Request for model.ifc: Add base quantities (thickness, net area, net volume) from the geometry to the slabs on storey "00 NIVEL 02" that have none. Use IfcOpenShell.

First a look at what the model holds.

```python
import ifcopenshell
import ifcopenshell.util.element
import ifcopenshell.util.unit

model = ifcopenshell.open("model.ifc")
print(model.schema)
for unit_type in ("LENGTHUNIT", "AREAUNIT", "VOLUMEUNIT"):
    print(unit_type, ifcopenshell.util.unit.calculate_unit_scale(model, unit_type))
storey = next(s for s in model.by_type("IfcBuildingStorey") if s.Name == "00 NIVEL 02")
slabs = [e for e in ifcopenshell.util.element.get_decomposition(storey) if e.is_a("IfcSlab")]
for e in sorted(slabs, key=lambda e: e.id()):
    print(e.id(), e.is_a(), e.Name, list(ifcopenshell.util.element.get_psets(e, qtos_only=True)), sep=" | ")
```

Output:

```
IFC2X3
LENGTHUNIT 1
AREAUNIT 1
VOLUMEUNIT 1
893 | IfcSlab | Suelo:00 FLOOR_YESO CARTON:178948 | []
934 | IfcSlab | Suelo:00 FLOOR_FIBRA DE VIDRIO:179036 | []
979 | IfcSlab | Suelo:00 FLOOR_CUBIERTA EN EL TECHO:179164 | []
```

```python
import ifcopenshell
import ifcopenshell.api.pset
import ifcopenshell.geom
import ifcopenshell.util.element
import ifcopenshell.util.shape
import ifcopenshell.util.unit

model = ifcopenshell.open("model.ifc")
unit_scale = ifcopenshell.util.unit.calculate_unit_scale(model)
area_scale = ifcopenshell.util.unit.calculate_unit_scale(model, "AREAUNIT")
volume_scale = ifcopenshell.util.unit.calculate_unit_scale(model, "VOLUMEUNIT")
settings = ifcopenshell.geom.settings()

storey = next(s for s in model.by_type("IfcBuildingStorey") if s.Name == "00 NIVEL 02")
slabs = [e for e in ifcopenshell.util.element.get_decomposition(storey) if e.is_a("IfcSlab")]

for e in sorted(slabs, key=lambda e: e.id()):
    if ifcopenshell.util.element.get_psets(e, qtos_only=True, should_inherit=False):
        continue
    # Geometry comes back in metres, in the element's own axes.
    shape = ifcopenshell.geom.create_shape(settings, e)
    values = {
        "Width": ifcopenshell.util.shape.get_z(shape.geometry) / unit_scale,
        "NetArea": ifcopenshell.util.shape.get_footprint_area(shape.geometry) / area_scale,
        "NetVolume": ifcopenshell.util.shape.get_volume(shape.geometry) / volume_scale,
    }
    qto = ifcopenshell.api.pset.add_qto(model, product=e, name="BaseQuantities")
    ifcopenshell.api.pset.edit_qto(model, qto=qto, properties=values)
    print(e.id(), {k: round(v, 3) for k, v in values.items()})

model.write("model_updated.ifc")
```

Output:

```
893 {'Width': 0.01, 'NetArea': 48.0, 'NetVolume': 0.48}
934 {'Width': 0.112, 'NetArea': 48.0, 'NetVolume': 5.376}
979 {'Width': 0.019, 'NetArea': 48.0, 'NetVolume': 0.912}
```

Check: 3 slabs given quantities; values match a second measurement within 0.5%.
